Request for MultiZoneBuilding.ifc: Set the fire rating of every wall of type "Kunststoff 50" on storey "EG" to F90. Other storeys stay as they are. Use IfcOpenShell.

First a look at what the model holds.

```python
import ifcopenshell
import ifcopenshell.util.element

model = ifcopenshell.open("MultiZoneBuilding.ifc")
print(model.schema)
storey = next(s for s in model.by_type("IfcBuildingStorey") if s.Name == "EG")
walls = [e for e in ifcopenshell.util.element.get_decomposition(storey) if e.is_a("IfcWall")]
seen = {}
for e in walls:
    element_type = ifcopenshell.util.element.get_type(e)
    key = (element_type.Name if element_type != e and element_type else None, ifcopenshell.util.element.get_pset(e, "Pset_WallCommon", "FireRating"))
    seen[key] = seen.get(key, 0) + 1
for (name, value), count in sorted(seen.items(), key=str):
    print(count, "x", name, "|", value)
```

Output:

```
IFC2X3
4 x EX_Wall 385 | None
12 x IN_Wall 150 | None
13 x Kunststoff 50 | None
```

```python
import ifcopenshell
import ifcopenshell.api.pset
import ifcopenshell.util.element

model = ifcopenshell.open("MultiZoneBuilding.ifc")

storey = next(s for s in model.by_type("IfcBuildingStorey") if s.Name == "EG")
walls = [e for e in ifcopenshell.util.element.get_decomposition(storey) if e.is_a("IfcWall")]

count = 0
for e in walls:
    element_type = ifcopenshell.util.element.get_type(e)
    if element_type in (None, e) or element_type.Name != "Kunststoff 50":
        continue
    # add_pset returns the element's existing set when there is one.
    pset = ifcopenshell.api.pset.add_pset(model, product=e, name="Pset_WallCommon")
    ifcopenshell.api.pset.edit_pset(model, pset=pset, properties={"FireRating": "F90"})
    count += 1

print(count, "walls updated")

model.write("MultiZoneBuilding_updated.ifc")
```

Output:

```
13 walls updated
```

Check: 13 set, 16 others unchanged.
